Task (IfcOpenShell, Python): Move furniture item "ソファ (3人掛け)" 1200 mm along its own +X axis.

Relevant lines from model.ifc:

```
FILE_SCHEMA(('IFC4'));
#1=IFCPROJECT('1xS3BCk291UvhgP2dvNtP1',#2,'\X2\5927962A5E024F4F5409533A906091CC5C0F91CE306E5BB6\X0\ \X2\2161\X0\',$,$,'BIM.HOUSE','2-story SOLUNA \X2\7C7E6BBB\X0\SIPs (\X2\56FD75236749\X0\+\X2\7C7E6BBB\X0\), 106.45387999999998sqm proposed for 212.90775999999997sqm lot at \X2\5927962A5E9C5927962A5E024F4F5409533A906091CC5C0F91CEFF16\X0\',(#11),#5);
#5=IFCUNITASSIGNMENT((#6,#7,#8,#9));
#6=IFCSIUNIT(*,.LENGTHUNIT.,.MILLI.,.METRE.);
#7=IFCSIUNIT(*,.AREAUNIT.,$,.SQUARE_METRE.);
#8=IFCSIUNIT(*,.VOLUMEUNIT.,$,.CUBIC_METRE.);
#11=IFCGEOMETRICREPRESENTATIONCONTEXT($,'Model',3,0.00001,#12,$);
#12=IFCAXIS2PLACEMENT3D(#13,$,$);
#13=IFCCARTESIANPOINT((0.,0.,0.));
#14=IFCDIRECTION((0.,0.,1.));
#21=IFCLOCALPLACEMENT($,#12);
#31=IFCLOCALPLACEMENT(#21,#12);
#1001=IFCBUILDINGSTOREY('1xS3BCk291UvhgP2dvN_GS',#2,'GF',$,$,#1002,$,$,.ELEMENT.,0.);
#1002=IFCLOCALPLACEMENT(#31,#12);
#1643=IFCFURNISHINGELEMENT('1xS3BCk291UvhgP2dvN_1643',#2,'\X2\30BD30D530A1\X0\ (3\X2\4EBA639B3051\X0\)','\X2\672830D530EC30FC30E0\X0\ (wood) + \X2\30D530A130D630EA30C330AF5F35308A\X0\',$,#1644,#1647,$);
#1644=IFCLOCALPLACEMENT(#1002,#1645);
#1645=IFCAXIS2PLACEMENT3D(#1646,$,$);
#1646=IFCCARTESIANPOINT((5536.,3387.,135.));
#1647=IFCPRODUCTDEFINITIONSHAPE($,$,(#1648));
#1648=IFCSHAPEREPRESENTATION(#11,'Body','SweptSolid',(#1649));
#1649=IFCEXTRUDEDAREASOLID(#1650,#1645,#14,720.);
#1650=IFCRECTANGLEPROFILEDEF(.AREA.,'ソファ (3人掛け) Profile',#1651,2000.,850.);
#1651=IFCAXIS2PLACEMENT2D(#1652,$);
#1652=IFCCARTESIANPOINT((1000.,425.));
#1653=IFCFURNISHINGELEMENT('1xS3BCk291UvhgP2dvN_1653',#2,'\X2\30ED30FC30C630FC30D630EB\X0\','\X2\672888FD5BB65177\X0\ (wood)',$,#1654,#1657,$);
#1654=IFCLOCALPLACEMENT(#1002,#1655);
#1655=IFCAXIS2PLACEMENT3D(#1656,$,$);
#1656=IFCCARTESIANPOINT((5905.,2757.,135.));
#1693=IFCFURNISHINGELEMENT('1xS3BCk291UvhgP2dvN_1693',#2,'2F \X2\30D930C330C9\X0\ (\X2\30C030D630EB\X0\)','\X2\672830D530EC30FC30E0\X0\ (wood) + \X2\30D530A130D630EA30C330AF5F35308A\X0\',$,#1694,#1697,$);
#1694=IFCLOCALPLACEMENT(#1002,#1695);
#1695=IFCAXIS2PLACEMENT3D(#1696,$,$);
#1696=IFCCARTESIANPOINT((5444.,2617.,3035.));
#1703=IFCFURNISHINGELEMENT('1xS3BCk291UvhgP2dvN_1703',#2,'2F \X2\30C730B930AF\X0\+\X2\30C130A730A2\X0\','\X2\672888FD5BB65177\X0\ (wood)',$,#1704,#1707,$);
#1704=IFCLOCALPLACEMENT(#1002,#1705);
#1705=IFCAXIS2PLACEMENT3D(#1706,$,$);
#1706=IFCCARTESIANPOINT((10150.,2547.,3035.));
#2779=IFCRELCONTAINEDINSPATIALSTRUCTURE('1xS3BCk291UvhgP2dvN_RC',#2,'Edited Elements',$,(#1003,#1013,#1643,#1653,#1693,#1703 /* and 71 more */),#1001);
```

```python
import ifcopenshell
import ifcopenshell.api.geometry
import ifcopenshell.util.placement
import ifcopenshell.util.unit

model = ifcopenshell.open("model.ifc")
unit_scale = ifcopenshell.util.unit.calculate_unit_scale(model)

item = model.by_guid("1xS3BCk291UvhgP2dvN_1643")
matrix = ifcopenshell.util.placement.get_local_placement(item.ObjectPlacement)
matrix[:3, 3] += matrix[:3, 0] * 1.2 / unit_scale
ifcopenshell.api.geometry.edit_object_placement(model, product=item, matrix=matrix, is_si=False)

print(ifcopenshell.util.placement.get_local_placement(item.ObjectPlacement).round(3) + 0.0)

model.write("model_rev.ifc")
```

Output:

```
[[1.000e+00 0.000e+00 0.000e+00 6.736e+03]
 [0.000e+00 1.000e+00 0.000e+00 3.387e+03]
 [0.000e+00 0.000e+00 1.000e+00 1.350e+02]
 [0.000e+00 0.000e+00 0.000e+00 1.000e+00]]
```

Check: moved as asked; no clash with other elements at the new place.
